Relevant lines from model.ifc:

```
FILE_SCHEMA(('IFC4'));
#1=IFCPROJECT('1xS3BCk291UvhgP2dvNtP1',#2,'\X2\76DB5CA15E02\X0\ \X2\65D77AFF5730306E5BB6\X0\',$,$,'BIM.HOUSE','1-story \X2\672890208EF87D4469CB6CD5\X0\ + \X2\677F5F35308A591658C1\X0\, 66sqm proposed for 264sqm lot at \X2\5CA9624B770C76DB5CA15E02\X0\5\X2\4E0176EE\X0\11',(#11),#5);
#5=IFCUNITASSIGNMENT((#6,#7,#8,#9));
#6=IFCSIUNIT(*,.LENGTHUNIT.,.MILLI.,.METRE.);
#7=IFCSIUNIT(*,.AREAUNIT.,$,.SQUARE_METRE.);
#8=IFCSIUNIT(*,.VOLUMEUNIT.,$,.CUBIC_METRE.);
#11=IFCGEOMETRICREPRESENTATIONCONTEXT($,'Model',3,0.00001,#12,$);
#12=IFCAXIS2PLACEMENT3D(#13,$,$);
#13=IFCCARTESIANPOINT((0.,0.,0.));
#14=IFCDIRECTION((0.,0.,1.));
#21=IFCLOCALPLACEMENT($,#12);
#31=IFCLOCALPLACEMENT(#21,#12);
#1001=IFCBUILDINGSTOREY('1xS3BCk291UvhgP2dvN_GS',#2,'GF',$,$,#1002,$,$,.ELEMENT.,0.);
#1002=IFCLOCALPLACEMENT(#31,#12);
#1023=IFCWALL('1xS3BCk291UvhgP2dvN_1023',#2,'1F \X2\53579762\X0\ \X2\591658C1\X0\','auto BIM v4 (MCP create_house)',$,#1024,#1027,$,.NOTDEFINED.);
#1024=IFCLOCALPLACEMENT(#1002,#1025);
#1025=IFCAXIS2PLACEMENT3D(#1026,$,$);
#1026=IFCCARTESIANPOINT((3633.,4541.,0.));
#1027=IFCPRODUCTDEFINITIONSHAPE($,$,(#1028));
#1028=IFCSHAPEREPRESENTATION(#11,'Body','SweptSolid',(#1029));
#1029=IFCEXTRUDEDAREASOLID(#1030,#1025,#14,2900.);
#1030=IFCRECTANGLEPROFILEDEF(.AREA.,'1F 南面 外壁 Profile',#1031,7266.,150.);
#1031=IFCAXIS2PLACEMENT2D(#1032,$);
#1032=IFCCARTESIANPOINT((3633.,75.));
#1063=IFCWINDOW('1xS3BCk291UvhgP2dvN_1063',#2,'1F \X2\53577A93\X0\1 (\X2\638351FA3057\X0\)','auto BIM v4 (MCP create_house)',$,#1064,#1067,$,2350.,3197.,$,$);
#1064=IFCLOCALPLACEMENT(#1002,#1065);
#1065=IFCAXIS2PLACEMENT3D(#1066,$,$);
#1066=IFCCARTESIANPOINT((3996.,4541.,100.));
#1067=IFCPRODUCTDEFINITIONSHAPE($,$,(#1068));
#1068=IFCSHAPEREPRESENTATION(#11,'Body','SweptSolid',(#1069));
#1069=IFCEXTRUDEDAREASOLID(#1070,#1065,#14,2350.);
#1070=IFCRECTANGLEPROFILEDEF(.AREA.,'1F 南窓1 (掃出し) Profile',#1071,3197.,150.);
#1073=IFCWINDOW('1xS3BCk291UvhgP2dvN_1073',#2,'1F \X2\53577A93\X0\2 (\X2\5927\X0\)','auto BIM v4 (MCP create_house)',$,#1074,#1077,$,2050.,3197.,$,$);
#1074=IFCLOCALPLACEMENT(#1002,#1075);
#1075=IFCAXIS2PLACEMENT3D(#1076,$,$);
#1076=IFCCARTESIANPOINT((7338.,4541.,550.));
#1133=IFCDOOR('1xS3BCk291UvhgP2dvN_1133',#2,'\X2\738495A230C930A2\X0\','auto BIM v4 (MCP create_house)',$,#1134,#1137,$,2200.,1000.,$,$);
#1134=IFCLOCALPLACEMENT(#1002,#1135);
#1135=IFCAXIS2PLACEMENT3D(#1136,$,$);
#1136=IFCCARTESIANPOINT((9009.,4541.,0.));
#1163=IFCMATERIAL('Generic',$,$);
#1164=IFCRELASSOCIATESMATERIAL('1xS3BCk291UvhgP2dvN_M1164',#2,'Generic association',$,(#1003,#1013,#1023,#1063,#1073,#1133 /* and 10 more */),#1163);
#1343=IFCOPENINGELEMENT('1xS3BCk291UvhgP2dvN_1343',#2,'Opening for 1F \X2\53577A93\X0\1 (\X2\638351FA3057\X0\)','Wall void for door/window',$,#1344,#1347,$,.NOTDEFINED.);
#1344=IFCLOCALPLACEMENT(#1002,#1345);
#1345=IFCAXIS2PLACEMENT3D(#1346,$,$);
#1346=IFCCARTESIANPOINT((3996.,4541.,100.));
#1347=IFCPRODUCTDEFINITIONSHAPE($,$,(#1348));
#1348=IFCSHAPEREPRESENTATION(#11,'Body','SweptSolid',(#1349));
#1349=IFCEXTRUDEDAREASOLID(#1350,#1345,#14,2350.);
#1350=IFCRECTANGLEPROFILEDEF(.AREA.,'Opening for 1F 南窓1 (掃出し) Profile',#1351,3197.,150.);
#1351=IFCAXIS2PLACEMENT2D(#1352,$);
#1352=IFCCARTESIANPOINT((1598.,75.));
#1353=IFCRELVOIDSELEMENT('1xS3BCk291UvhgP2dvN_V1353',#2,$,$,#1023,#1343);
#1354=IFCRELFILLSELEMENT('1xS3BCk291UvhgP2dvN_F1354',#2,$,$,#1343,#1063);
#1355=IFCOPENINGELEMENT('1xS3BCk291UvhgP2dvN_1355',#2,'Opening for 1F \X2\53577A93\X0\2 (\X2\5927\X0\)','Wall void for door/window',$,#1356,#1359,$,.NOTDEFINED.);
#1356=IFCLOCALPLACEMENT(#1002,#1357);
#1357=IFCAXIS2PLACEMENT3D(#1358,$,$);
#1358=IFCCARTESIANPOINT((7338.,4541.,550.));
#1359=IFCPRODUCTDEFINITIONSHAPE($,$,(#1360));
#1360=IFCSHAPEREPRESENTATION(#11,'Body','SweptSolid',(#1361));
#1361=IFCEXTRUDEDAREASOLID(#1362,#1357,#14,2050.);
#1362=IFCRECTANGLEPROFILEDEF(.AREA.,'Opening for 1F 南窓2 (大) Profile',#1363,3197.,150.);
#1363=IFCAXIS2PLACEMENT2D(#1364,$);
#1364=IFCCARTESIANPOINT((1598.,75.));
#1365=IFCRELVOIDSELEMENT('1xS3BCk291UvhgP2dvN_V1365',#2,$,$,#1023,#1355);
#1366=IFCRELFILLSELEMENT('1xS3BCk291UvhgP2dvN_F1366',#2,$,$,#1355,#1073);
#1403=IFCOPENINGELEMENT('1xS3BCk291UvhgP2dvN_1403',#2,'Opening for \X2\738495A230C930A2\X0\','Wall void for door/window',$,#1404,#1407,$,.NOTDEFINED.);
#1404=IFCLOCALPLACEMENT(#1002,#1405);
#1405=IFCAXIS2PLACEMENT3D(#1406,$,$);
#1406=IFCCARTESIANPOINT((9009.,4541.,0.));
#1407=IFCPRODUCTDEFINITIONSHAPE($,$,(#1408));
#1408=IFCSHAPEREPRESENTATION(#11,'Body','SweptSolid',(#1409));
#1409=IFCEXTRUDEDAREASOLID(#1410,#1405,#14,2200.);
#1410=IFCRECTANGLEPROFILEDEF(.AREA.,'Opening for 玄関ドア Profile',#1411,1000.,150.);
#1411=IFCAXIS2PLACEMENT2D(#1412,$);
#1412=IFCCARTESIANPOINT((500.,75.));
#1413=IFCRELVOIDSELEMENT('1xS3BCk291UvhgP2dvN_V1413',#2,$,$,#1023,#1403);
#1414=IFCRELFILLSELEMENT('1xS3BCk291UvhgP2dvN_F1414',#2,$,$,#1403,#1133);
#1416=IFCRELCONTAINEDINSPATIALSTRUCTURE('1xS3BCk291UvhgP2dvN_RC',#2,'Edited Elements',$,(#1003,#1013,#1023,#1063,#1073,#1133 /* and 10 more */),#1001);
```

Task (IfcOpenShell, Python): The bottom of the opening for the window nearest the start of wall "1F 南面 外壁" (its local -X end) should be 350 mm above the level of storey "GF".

```python
import numpy as np
import ifcopenshell
import ifcopenshell.api.geometry
import ifcopenshell.geom
import ifcopenshell.util.element
import ifcopenshell.util.placement
import ifcopenshell.util.shape
import ifcopenshell.util.unit

model = ifcopenshell.open("model.ifc")
unit_scale = ifcopenshell.util.unit.calculate_unit_scale(model)

window = model.by_guid("1xS3BCk291UvhgP2dvN_1063")
opening = window.FillsVoids[0].RelatingOpeningElement
storey = ifcopenshell.util.element.get_container(window, ifc_class="IfcBuildingStorey")
level = ifcopenshell.util.placement.get_local_placement(storey.ObjectPlacement)[2, 3]

# The opening's origin need not be at the sill, so measure its lowest point.
shape = ifcopenshell.geom.create_shape(ifcopenshell.geom.settings(), opening)
bottom = ifcopenshell.util.shape.get_shape_bottom_elevation(shape, shape.geometry) / unit_scale
dz = level + 350.0 - bottom

shift = np.array([0.0, 0.0, dz])
# The window is not placed relative to its opening, so move both.
for product in (opening, window):
    matrix = ifcopenshell.util.placement.get_local_placement(product.ObjectPlacement)
    matrix[:3, 3] += shift
    ifcopenshell.api.geometry.edit_object_placement(model, product=product, matrix=matrix, is_si=False)

print(f"moved by {dz * unit_scale:+.3f} m")

model.write("model_updated.ifc")
```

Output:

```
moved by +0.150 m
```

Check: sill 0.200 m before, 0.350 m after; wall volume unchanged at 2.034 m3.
